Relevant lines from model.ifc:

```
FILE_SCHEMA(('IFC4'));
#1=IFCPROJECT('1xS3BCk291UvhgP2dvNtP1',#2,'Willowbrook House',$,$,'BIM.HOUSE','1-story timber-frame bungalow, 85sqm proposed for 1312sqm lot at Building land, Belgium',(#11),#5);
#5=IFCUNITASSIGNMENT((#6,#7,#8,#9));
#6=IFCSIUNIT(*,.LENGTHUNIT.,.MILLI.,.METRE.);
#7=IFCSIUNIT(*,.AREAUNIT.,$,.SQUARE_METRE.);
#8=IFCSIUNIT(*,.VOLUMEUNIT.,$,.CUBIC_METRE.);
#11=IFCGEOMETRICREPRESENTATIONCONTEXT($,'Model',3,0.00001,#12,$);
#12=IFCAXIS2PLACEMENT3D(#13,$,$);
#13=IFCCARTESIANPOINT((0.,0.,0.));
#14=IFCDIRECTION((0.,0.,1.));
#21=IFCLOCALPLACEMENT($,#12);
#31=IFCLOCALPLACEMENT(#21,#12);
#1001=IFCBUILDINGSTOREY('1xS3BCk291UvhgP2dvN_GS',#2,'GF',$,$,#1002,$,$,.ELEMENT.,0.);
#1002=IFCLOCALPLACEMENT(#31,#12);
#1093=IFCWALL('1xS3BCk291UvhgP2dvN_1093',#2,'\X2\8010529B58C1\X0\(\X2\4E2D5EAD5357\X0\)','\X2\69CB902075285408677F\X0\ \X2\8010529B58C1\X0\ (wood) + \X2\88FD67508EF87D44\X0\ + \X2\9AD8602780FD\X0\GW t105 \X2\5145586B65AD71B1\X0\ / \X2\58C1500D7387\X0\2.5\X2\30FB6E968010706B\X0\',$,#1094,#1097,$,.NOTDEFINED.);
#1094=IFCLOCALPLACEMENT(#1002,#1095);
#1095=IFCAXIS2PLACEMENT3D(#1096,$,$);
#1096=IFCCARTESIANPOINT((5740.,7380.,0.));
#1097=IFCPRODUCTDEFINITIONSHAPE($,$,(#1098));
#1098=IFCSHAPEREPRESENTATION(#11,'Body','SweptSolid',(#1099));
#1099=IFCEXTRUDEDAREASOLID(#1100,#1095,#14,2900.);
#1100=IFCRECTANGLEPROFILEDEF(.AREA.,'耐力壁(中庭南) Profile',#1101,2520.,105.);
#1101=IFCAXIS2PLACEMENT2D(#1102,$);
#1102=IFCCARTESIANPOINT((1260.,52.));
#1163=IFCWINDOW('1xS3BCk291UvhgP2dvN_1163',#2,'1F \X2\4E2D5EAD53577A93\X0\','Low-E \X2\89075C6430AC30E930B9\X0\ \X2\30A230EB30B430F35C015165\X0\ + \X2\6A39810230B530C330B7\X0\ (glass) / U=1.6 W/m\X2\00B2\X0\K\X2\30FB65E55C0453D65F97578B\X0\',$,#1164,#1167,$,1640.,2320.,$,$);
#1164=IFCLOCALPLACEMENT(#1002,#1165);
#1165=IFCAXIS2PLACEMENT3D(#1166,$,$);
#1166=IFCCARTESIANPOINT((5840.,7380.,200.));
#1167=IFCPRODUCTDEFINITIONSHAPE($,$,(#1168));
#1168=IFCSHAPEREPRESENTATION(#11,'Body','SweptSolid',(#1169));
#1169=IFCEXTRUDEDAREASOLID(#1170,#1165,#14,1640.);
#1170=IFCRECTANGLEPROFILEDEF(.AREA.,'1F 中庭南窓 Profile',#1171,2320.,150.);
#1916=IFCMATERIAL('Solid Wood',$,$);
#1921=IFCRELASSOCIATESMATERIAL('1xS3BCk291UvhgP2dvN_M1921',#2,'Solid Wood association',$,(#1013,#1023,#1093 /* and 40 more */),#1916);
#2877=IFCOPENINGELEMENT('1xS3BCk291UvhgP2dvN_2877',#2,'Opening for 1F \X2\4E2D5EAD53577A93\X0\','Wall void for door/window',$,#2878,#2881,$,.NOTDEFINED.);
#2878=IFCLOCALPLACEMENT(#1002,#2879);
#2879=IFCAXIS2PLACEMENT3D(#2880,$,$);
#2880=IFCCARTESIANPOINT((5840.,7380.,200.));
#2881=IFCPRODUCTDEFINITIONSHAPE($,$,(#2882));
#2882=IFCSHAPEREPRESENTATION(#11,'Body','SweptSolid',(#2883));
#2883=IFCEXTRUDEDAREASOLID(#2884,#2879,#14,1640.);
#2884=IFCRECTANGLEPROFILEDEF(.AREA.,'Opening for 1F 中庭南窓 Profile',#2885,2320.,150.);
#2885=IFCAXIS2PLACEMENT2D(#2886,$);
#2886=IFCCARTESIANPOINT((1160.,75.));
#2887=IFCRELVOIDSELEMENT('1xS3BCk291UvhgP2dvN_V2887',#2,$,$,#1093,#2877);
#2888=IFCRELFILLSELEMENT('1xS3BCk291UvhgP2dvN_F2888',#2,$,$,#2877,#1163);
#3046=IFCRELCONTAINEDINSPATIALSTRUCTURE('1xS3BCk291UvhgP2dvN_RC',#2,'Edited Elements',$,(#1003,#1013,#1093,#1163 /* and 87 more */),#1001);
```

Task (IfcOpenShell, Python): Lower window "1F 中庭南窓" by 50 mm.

```python
import numpy as np
import ifcopenshell
import ifcopenshell.api.geometry
import ifcopenshell.util.placement
import ifcopenshell.util.unit

model = ifcopenshell.open("model.ifc")
unit_scale = ifcopenshell.util.unit.calculate_unit_scale(model)

window = model.by_guid("1xS3BCk291UvhgP2dvN_1163")
opening = window.FillsVoids[0].RelatingOpeningElement
dz = -0.05 / unit_scale

shift = np.array([0.0, 0.0, dz])
# The window is not placed relative to its opening, so move both.
for product in (opening, window):
    matrix = ifcopenshell.util.placement.get_local_placement(product.ObjectPlacement)
    matrix[:3, 3] += shift
    ifcopenshell.api.geometry.edit_object_placement(model, product=product, matrix=matrix, is_si=False)

print(f"moved by {dz * unit_scale:+.3f} m")

model.write("model-out.ifc")
```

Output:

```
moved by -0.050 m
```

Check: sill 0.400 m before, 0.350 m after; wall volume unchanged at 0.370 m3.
